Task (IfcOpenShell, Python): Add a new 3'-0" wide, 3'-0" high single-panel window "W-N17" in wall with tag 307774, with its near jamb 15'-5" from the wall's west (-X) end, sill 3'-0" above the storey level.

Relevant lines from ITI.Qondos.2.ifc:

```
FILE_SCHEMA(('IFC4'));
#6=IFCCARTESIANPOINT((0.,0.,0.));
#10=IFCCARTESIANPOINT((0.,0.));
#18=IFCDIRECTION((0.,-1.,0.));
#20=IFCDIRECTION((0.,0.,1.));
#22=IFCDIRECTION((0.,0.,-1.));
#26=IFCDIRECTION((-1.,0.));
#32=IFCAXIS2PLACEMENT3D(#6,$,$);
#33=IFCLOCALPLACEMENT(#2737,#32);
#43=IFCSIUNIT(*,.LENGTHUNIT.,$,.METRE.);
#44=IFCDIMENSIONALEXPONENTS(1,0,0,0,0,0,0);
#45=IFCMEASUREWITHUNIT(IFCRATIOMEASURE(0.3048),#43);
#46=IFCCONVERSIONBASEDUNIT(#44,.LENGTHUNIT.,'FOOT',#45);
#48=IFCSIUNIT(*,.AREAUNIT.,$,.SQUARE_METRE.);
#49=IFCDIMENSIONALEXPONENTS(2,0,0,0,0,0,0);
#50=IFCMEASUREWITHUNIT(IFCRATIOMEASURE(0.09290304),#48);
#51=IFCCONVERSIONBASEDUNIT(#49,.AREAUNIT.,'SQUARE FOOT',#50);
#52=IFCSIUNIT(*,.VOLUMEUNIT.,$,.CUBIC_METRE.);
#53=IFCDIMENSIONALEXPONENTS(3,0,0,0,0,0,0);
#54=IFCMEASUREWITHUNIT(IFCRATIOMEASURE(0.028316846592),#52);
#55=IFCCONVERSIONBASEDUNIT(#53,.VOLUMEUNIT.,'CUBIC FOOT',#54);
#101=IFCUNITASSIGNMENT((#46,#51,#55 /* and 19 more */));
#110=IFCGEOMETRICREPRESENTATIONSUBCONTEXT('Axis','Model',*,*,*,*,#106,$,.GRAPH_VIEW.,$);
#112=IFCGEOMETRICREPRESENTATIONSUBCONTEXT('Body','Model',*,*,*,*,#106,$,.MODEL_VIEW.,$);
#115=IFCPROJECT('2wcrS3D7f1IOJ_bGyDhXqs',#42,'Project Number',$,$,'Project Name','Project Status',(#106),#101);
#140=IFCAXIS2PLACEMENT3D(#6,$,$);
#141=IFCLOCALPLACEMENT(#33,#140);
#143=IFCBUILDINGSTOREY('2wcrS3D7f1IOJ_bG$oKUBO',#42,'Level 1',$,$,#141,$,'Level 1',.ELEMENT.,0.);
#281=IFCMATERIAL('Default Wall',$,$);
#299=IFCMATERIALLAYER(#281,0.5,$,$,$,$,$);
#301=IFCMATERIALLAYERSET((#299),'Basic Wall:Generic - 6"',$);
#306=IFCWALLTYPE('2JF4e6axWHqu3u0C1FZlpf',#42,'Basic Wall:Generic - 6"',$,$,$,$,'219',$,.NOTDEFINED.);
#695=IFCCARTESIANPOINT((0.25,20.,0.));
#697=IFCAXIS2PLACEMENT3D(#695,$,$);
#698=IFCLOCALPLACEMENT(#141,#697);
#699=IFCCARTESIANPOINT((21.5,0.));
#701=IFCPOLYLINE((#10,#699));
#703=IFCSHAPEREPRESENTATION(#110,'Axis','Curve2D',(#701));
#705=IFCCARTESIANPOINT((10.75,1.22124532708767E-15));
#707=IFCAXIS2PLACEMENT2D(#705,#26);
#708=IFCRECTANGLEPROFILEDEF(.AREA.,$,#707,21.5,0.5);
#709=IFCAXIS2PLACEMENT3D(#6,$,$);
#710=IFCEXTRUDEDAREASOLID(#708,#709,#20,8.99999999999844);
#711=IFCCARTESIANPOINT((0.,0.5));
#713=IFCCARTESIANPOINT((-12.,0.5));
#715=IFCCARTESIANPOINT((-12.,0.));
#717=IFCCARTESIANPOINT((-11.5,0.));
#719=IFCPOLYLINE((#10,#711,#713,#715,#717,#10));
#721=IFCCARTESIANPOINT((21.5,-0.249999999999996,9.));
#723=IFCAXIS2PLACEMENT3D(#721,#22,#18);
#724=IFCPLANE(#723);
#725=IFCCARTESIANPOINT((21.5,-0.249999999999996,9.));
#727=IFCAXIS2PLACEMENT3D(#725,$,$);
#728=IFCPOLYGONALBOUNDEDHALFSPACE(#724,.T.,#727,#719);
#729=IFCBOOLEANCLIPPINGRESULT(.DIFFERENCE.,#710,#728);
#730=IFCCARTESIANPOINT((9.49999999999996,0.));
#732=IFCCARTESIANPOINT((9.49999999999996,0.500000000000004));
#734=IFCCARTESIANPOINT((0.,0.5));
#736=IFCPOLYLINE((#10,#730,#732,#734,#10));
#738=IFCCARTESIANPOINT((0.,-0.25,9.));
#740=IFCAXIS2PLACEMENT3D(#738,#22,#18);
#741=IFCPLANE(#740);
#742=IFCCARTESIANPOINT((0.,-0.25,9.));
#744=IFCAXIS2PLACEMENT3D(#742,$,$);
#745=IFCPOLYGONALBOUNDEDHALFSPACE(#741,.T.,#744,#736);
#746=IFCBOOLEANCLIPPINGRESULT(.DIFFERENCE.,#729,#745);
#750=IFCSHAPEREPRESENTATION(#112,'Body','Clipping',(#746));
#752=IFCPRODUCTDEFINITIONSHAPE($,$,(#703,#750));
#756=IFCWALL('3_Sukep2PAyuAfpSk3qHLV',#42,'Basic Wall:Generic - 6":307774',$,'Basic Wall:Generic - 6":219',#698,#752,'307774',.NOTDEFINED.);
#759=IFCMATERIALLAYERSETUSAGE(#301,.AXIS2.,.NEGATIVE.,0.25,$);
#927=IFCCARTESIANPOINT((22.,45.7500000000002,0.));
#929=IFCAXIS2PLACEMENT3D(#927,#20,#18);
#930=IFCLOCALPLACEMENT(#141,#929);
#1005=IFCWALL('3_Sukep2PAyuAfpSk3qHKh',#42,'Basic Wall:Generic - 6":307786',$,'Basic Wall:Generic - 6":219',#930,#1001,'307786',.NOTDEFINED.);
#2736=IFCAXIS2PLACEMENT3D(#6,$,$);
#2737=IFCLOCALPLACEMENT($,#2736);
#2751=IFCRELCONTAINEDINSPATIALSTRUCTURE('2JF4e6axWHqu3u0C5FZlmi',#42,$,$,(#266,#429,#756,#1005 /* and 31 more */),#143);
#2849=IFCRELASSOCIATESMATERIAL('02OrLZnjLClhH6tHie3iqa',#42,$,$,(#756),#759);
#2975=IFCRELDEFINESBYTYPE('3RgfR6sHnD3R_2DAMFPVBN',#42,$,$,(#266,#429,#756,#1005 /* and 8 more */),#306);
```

```python
import numpy as np
import ifcopenshell
import ifcopenshell.api.feature
import ifcopenshell.api.geometry
import ifcopenshell.api.root
import ifcopenshell.api.spatial
import ifcopenshell.geom
import ifcopenshell.util.element
import ifcopenshell.util.placement
import ifcopenshell.util.representation
import ifcopenshell.util.shape
import ifcopenshell.util.unit

model = ifcopenshell.open("ITI.Qondos.2.ifc")
unit_scale = ifcopenshell.util.unit.calculate_unit_scale(model)
settings = ifcopenshell.geom.settings()


def volume(element):
    """Net volume in cubic metres, openings subtracted."""
    shape = ifcopenshell.geom.create_shape(settings, element)
    return ifcopenshell.util.shape.get_volume(shape.geometry)


wall = model.by_guid("3_Sukep2PAyuAfpSk3qHLV")
storey = ifcopenshell.util.element.get_container(wall, ifc_class="IfcBuildingStorey")
context = ifcopenshell.util.representation.get_context(model, "Model", "Body", "MODEL_VIEW")
before = volume(wall)

width, height, from_end, sill = 0.9144, 0.9144, 4.699, 0.9144  # metres

# The wall runs along its own X axis, and the end named is its -X end.
wall_shape = ifcopenshell.geom.create_shape(settings, wall)
x, y, z = ifcopenshell.util.shape.get_vertices(wall_shape.geometry).T
start = x.min() + from_end
face, thickness = float(y.min()), float(y.max() - y.min())
wall_matrix = ifcopenshell.util.placement.get_local_placement(wall.ObjectPlacement)
level = ifcopenshell.util.placement.get_local_placement(storey.ObjectPlacement)[2, 3]


def in_wall(x, y):
    """Placement at x, y metres in the wall's axes, at sill height."""
    matrix = wall_matrix.copy()
    matrix[:, 3] = wall_matrix @ np.array([x / unit_scale, y / unit_scale, 0.0, 1.0])
    matrix[2, 3] = level + sill / unit_scale
    return matrix


# Opening: a box that overshoots both wall faces by 50 mm.
opening = ifcopenshell.api.root.create_entity(model, ifc_class="IfcOpeningElement", predefined_type="OPENING")
box = ifcopenshell.api.geometry.add_wall_representation(
    model, context=context, length=width, height=height, thickness=thickness + 0.1
)
ifcopenshell.api.geometry.assign_representation(model, product=opening, representation=box)
ifcopenshell.api.geometry.edit_object_placement(model, product=opening, matrix=in_wall(start, face - 0.05), is_si=False)
ifcopenshell.api.feature.add_feature(model, feature=opening, element=wall)

window = ifcopenshell.api.root.create_entity(model, ifc_class="IfcWindow", name="W-N17", predefined_type="WINDOW")
window.OverallWidth, window.OverallHeight = width / unit_scale, height / unit_scale
window.PartitioningType = "SINGLE_PANEL"
body = ifcopenshell.api.geometry.add_window_representation(
    model,
    context=context,
    overall_width=window.OverallWidth,
    overall_height=window.OverallHeight,
    partition_type="SINGLE_PANEL",
)
ifcopenshell.api.geometry.assign_representation(model, product=window, representation=body)
ifcopenshell.api.spatial.assign_container(model, products=[window], relating_structure=storey)
ifcopenshell.api.feature.add_filling(model, opening=opening, element=window)

# Centre the window in the wall's thickness.
ifcopenshell.api.geometry.edit_object_placement(model, product=window, matrix=in_wall(start, face), is_si=False)
window_shape = ifcopenshell.geom.create_shape(settings, window)
depth = ifcopenshell.util.shape.get_vertices(window_shape.geometry)[:, 1]
offset = face + thickness / 2 - (depth.min() + depth.max()) / 2
ifcopenshell.api.geometry.edit_object_placement(model, product=window, matrix=in_wall(start, offset), is_si=False)

after = volume(wall)

print(f"wall volume {before:.3f} -> {after:.3f} m3")

model.write("ITI.Qondos.2_v2.ifc")
```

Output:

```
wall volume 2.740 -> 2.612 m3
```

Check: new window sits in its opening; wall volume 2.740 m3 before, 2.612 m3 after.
